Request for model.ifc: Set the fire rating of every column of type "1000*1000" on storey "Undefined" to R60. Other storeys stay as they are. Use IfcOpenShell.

First a look at what the model holds.

```python
import ifcopenshell
import ifcopenshell.util.element

model = ifcopenshell.open("model.ifc")
print(model.schema)
storey = next(s for s in model.by_type("IfcBuildingStorey") if s.Name == "Undefined")
columns = [e for e in ifcopenshell.util.element.get_decomposition(storey) if e.is_a("IfcColumn")]
seen = {}
for e in columns:
    element_type = ifcopenshell.util.element.get_type(e)
    key = (element_type.Name if element_type != e and element_type else None, ifcopenshell.util.element.get_pset(e, "Pset_ColumnCommon", "FireRating"))
    seen[key] = seen.get(key, 0) + 1
for (name, value), count in sorted(seen.items(), key=str):
    print(count, "x", name, "|", value)
```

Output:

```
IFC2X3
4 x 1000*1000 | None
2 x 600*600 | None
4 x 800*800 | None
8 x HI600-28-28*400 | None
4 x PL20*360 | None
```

```python
import ifcopenshell
import ifcopenshell.api.pset
import ifcopenshell.util.element

model = ifcopenshell.open("model.ifc")

storey = next(s for s in model.by_type("IfcBuildingStorey") if s.Name == "Undefined")
columns = [e for e in ifcopenshell.util.element.get_decomposition(storey) if e.is_a("IfcColumn")]

count = 0
for e in columns:
    element_type = ifcopenshell.util.element.get_type(e)
    if element_type in (None, e) or element_type.Name != "1000*1000":
        continue
    found = ifcopenshell.util.element.get_pset(e, "Pset_ColumnCommon", should_inherit=False)
    if found:
        pset = model.by_id(found["id"])
        if len(ifcopenshell.util.element.get_elements_by_pset(pset)) > 1:
            pset = ifcopenshell.api.pset.unshare_pset(model, products=[e], pset=pset)[0]
    else:
        pset = ifcopenshell.api.pset.add_pset(model, product=e, name="Pset_ColumnCommon")
    ifcopenshell.api.pset.edit_pset(model, pset=pset, properties={"FireRating": "R60"})
    count += 1

print(count, "columns updated")

model.write("model-out.ifc")
```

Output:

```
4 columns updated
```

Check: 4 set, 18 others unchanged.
